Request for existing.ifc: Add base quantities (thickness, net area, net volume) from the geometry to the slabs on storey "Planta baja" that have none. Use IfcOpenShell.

First a look at what the model holds.

```python
import ifcopenshell
import ifcopenshell.util.element
import ifcopenshell.util.unit

model = ifcopenshell.open("existing.ifc")
print(model.schema)
for unit_type in ("LENGTHUNIT", "AREAUNIT", "VOLUMEUNIT"):
    print(unit_type, ifcopenshell.util.unit.calculate_unit_scale(model, unit_type))
storey = next(s for s in model.by_type("IfcBuildingStorey") if s.Name == "Planta baja")
slabs = [e for e in ifcopenshell.util.element.get_decomposition(storey) if e.is_a("IfcSlab")]
for e in sorted(slabs, key=lambda e: e.id()):
    print(e.id(), e.is_a(), e.Name, list(ifcopenshell.util.element.get_psets(e, qtos_only=True)), sep=" | ")
```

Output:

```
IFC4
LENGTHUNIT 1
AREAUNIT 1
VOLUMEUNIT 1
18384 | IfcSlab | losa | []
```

```python
import ifcopenshell
import ifcopenshell.api.pset
import ifcopenshell.geom
import ifcopenshell.util.element
import ifcopenshell.util.shape
import ifcopenshell.util.unit

model = ifcopenshell.open("existing.ifc")
unit_scale = ifcopenshell.util.unit.calculate_unit_scale(model)
area_scale = ifcopenshell.util.unit.calculate_unit_scale(model, "AREAUNIT")
volume_scale = ifcopenshell.util.unit.calculate_unit_scale(model, "VOLUMEUNIT")
settings = ifcopenshell.geom.settings()

storey = next(s for s in model.by_type("IfcBuildingStorey") if s.Name == "Planta baja")
slabs = [e for e in ifcopenshell.util.element.get_decomposition(storey) if e.is_a("IfcSlab")]

for e in sorted(slabs, key=lambda e: e.id()):
    if ifcopenshell.util.element.get_psets(e, qtos_only=True, should_inherit=False):
        continue
    # Geometry comes back in metres, in the element's own axes.
    shape = ifcopenshell.geom.create_shape(settings, e)
    values = {
        "Width": ifcopenshell.util.shape.get_z(shape.geometry) / unit_scale,
        "NetArea": ifcopenshell.util.shape.get_footprint_area(shape.geometry) / area_scale,
        "NetVolume": ifcopenshell.util.shape.get_volume(shape.geometry) / volume_scale,
    }
    qto = ifcopenshell.api.pset.add_qto(model, product=e, name="Qto_SlabBaseQuantities")
    ifcopenshell.api.pset.edit_qto(model, qto=qto, properties=values)
    print(e.id(), {k: round(v, 3) for k, v in values.items()})

model.write("existing_v2.ifc")
```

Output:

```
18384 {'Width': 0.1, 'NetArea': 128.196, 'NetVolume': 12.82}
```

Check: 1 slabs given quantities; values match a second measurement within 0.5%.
